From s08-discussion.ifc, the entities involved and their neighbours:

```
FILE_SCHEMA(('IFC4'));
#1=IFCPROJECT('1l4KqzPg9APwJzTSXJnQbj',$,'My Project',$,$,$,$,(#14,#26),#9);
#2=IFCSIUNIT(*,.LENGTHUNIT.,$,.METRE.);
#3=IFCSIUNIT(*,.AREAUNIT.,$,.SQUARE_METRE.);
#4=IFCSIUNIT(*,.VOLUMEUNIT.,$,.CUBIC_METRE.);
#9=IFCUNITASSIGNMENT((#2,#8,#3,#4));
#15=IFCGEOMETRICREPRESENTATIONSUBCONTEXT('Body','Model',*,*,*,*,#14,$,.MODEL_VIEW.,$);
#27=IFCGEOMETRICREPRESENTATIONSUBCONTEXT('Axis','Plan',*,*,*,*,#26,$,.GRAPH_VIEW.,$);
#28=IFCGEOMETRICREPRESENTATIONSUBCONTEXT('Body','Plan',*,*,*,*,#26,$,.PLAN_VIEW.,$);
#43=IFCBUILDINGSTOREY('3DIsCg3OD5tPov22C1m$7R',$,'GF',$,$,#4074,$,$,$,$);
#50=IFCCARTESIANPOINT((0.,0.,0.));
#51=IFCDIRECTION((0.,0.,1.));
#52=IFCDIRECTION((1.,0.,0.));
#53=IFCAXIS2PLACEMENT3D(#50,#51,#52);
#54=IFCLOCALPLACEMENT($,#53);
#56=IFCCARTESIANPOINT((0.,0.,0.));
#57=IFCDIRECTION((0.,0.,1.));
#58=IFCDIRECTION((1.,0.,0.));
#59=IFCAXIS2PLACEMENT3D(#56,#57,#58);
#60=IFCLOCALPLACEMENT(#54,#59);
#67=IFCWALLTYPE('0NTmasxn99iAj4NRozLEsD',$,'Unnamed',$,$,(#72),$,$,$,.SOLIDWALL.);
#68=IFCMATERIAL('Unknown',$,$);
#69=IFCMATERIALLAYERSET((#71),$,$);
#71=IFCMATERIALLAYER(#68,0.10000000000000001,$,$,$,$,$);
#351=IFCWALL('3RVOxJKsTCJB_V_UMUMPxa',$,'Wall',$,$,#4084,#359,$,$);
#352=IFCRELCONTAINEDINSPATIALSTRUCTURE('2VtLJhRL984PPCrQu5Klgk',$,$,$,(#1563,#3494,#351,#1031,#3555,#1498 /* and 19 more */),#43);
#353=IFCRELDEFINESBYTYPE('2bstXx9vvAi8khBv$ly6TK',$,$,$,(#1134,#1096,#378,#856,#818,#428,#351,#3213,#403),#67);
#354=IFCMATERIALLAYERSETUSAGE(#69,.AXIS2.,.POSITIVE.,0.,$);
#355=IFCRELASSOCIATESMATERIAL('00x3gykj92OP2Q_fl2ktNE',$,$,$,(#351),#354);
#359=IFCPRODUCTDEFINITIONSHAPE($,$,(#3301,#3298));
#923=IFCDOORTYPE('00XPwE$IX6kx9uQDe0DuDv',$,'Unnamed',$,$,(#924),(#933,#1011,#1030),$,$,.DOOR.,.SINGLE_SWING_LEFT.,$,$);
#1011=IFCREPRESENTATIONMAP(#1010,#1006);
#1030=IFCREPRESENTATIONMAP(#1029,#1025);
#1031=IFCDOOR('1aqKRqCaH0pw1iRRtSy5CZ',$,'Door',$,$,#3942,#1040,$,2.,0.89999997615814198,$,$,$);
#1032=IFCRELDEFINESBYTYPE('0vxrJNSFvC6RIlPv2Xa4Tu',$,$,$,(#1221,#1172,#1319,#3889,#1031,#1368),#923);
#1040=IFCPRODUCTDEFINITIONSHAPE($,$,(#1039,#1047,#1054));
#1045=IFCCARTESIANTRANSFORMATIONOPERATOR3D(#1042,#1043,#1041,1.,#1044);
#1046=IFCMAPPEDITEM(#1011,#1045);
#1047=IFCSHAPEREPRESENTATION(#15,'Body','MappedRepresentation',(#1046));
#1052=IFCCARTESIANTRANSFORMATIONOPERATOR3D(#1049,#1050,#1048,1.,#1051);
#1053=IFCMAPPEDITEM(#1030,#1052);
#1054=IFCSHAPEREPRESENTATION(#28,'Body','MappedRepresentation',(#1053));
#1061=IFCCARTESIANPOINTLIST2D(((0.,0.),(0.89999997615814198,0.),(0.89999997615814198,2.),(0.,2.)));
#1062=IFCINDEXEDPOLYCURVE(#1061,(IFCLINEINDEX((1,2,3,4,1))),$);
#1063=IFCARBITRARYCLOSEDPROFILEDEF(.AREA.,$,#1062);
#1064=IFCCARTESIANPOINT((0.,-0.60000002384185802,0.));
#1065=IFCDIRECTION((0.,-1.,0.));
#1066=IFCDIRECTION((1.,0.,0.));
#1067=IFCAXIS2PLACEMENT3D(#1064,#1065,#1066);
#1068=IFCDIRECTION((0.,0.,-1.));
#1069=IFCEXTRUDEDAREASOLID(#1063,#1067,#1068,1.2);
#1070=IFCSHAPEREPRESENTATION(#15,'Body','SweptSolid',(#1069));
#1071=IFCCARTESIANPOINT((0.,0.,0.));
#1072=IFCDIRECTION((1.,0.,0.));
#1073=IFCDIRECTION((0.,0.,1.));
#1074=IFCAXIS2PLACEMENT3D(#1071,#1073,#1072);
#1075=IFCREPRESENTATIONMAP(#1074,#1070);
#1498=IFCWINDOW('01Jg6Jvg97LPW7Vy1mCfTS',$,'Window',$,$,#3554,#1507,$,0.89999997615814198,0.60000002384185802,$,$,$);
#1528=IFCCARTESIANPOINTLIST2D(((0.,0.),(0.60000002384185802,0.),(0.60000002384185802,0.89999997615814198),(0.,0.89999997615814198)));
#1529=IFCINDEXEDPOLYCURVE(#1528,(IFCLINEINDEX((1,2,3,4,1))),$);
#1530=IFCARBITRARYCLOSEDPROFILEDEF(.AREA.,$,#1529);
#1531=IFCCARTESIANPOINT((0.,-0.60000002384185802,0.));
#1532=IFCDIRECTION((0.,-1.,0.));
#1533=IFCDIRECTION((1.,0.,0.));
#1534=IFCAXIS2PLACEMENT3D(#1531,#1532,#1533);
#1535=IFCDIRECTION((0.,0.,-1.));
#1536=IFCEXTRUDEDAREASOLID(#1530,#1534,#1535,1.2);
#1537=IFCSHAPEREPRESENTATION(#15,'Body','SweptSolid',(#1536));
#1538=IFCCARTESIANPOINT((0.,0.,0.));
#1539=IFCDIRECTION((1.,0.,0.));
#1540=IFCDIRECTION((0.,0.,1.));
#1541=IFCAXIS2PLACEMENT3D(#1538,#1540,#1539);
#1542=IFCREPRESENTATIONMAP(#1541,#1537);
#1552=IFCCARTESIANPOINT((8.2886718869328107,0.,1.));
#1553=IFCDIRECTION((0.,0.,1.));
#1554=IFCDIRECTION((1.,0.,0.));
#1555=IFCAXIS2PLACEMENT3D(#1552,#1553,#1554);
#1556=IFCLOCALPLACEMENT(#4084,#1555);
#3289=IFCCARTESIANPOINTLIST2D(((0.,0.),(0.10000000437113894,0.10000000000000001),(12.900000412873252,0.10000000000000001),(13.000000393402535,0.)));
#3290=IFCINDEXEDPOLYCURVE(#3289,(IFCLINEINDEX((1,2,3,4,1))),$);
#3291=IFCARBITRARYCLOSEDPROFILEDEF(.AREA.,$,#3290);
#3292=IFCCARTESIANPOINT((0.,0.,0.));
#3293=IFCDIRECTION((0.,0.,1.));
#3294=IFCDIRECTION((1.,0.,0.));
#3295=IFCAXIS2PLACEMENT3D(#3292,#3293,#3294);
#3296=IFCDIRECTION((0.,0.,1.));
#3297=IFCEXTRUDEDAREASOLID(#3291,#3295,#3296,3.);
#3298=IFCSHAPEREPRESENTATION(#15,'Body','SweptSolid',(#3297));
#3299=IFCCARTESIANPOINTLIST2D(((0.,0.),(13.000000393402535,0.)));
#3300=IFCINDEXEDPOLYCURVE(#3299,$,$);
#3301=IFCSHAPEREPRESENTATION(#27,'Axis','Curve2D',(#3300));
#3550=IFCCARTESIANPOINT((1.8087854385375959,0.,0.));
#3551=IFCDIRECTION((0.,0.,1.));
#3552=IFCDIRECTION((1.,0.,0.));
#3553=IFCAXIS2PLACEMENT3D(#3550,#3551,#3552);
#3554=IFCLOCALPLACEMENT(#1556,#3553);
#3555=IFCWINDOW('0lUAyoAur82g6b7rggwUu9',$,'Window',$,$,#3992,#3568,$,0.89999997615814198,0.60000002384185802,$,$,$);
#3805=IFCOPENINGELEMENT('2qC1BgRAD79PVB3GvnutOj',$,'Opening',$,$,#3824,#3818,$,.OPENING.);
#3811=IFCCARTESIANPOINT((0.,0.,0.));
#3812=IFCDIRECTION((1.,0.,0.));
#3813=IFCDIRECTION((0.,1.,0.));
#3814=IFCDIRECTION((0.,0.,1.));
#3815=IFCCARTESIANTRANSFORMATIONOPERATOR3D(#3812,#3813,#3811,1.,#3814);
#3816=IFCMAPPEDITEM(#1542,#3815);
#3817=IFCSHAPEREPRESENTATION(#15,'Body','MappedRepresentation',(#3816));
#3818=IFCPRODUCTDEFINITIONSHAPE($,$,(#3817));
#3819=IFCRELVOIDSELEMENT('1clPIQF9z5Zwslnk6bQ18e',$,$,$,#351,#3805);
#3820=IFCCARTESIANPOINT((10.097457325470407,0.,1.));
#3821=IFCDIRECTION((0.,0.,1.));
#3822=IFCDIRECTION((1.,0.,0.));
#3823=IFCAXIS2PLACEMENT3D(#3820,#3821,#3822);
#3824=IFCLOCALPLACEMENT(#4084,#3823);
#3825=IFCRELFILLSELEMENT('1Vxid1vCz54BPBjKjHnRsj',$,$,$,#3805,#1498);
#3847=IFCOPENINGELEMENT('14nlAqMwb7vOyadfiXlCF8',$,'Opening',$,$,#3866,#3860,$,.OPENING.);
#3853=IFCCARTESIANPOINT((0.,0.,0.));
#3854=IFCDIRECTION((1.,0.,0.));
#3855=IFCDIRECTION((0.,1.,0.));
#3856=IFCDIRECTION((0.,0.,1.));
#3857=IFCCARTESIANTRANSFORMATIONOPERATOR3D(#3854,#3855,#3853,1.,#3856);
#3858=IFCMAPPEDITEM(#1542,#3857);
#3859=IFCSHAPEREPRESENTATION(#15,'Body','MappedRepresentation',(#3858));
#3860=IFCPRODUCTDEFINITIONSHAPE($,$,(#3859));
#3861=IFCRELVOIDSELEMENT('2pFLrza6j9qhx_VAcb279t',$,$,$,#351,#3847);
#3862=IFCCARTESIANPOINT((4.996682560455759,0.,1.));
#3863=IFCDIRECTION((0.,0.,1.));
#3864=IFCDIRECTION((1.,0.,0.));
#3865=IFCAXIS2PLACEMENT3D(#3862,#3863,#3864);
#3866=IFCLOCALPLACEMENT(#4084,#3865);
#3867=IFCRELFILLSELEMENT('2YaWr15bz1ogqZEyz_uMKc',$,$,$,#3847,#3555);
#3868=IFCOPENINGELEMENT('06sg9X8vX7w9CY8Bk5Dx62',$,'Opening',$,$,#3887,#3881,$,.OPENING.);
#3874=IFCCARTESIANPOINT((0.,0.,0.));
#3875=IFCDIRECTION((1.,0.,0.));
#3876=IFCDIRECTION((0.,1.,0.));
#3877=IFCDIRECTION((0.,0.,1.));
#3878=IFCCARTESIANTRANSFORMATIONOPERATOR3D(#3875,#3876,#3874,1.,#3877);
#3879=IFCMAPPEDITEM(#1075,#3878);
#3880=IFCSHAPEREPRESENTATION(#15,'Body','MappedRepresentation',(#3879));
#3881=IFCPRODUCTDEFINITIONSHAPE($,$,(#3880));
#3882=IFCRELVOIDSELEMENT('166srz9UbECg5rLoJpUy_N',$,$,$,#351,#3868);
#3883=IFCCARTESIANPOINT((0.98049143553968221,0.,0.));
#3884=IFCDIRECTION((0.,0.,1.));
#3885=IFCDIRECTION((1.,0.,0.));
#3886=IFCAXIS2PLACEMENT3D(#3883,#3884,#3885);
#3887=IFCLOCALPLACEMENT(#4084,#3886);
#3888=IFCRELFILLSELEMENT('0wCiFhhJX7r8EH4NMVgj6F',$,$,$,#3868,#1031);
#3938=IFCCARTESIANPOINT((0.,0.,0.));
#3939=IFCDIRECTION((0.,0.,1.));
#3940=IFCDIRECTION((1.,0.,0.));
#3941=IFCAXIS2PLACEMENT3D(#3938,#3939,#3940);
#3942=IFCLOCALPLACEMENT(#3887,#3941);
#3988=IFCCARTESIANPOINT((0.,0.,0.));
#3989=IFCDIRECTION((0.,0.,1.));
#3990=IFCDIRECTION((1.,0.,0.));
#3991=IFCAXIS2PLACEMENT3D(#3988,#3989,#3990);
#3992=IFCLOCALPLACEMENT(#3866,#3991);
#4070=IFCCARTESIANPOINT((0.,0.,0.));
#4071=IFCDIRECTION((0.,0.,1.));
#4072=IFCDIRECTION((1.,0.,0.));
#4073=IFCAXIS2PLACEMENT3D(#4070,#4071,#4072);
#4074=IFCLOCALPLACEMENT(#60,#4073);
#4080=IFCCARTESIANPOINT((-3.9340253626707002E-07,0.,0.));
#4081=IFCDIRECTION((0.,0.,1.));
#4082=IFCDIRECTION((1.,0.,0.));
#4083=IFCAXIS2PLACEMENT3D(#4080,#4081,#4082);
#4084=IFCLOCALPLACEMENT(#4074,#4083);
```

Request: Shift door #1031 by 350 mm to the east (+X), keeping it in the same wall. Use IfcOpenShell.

```python
import ifcopenshell
import ifcopenshell.api.geometry
import ifcopenshell.util.placement
import ifcopenshell.util.unit

model = ifcopenshell.open("s08-discussion.ifc")
unit_scale = ifcopenshell.util.unit.calculate_unit_scale(model)

door = model.by_id(1031)
opening = door.FillsVoids[0].RelatingOpeningElement
wall = opening.VoidsElements[0].RelatingBuildingElement

wall_matrix = ifcopenshell.util.placement.get_local_placement(wall.ObjectPlacement)
shift = wall_matrix[:3, 0] * 0.35 / unit_scale
before = ifcopenshell.util.placement.get_local_placement(door.ObjectPlacement)[:3, 3].copy()

# The door is placed relative to its opening, so it follows when the opening moves.
matrix = ifcopenshell.util.placement.get_local_placement(opening.ObjectPlacement)
matrix[:3, 3] += shift
ifcopenshell.api.geometry.edit_object_placement(
    model, product=opening, matrix=matrix, is_si=False, should_transform_children=True
)

after = ifcopenshell.util.placement.get_local_placement(door.ObjectPlacement)[:3, 3]
print("door moved by", (after - before).round(3) + 0.0)

model.write("s08-discussion_v2.ifc")
```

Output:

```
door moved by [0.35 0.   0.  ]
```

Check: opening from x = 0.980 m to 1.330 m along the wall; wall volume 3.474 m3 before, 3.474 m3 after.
